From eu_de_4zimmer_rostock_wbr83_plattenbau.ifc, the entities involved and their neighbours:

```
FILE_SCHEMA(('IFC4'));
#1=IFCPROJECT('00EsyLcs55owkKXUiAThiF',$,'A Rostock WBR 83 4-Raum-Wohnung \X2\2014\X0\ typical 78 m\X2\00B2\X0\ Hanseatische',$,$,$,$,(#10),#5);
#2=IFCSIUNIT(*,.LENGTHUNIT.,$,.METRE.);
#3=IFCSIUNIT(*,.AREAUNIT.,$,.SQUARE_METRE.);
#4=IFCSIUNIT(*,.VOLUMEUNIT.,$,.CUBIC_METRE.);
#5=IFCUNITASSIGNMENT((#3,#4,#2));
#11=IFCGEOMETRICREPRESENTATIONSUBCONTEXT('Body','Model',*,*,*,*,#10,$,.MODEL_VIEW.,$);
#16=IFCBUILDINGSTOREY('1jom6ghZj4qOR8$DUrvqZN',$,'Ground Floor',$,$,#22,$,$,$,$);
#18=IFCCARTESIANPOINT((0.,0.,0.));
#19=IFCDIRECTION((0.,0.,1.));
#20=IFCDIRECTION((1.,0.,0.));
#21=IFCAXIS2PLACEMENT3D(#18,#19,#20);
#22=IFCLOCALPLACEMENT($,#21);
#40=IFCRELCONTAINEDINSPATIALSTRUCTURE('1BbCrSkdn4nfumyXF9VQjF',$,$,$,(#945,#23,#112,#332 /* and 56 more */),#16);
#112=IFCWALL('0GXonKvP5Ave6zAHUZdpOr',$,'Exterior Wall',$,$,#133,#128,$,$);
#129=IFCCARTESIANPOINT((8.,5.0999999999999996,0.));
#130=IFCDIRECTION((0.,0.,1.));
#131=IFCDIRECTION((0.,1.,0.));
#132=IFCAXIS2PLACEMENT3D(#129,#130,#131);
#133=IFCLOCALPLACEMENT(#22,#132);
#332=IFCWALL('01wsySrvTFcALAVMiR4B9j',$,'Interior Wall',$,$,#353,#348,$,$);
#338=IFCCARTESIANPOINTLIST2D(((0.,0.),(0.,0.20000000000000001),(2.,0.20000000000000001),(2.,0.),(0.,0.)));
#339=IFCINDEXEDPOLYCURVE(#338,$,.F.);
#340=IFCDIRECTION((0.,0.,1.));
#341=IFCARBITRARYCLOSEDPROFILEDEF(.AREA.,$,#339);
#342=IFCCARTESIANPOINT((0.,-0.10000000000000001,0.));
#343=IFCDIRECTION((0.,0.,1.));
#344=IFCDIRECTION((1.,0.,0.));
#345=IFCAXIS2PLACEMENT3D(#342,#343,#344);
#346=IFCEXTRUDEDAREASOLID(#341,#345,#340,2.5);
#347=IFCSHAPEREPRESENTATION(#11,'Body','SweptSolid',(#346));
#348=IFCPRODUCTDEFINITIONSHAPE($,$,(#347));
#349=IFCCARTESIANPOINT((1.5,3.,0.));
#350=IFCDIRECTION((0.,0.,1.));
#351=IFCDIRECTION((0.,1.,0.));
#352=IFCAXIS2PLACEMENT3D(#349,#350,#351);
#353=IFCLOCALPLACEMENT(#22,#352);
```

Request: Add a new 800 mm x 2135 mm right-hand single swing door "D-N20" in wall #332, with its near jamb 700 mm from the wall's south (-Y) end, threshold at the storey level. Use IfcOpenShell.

```python
import numpy as np
import ifcopenshell
import ifcopenshell.api.feature
import ifcopenshell.api.geometry
import ifcopenshell.api.root
import ifcopenshell.api.spatial
import ifcopenshell.geom
import ifcopenshell.util.element
import ifcopenshell.util.placement
import ifcopenshell.util.representation
import ifcopenshell.util.shape
import ifcopenshell.util.unit

model = ifcopenshell.open("eu_de_4zimmer_rostock_wbr83_plattenbau.ifc")
unit_scale = ifcopenshell.util.unit.calculate_unit_scale(model)
settings = ifcopenshell.geom.settings()


def volume(element):
    """Net volume in cubic metres, openings subtracted."""
    shape = ifcopenshell.geom.create_shape(settings, element)
    return ifcopenshell.util.shape.get_volume(shape.geometry)


wall = model.by_guid("01wsySrvTFcALAVMiR4B9j")
storey = ifcopenshell.util.element.get_container(wall, ifc_class="IfcBuildingStorey")
context = ifcopenshell.util.representation.get_context(model, "Model", "Body", "MODEL_VIEW")
before = volume(wall)

width, height, from_end, sill = 0.8, 2.135, 0.7, 0.0  # metres

# The wall runs along its own X axis, and the end named is its -X end.
wall_shape = ifcopenshell.geom.create_shape(settings, wall)
x, y, z = ifcopenshell.util.shape.get_vertices(wall_shape.geometry).T
start = x.min() + from_end
face, thickness = float(y.min()), float(y.max() - y.min())
wall_matrix = ifcopenshell.util.placement.get_local_placement(wall.ObjectPlacement)
level = ifcopenshell.util.placement.get_local_placement(storey.ObjectPlacement)[2, 3]


def in_wall(x, y):
    """Placement at x, y metres in the wall's axes, at sill height."""
    matrix = wall_matrix.copy()
    matrix[:, 3] = wall_matrix @ np.array([x / unit_scale, y / unit_scale, 0.0, 1.0])
    matrix[2, 3] = level + sill / unit_scale
    return matrix


# Opening: a box that overshoots both wall faces by 50 mm.
opening = ifcopenshell.api.root.create_entity(model, ifc_class="IfcOpeningElement", predefined_type="OPENING")
box = ifcopenshell.api.geometry.add_wall_representation(
    model, context=context, length=width, height=height, thickness=thickness + 0.1
)
ifcopenshell.api.geometry.assign_representation(model, product=opening, representation=box)
ifcopenshell.api.geometry.edit_object_placement(model, product=opening, matrix=in_wall(start, face - 0.05), is_si=False)
ifcopenshell.api.feature.add_feature(model, feature=opening, element=wall)

door = ifcopenshell.api.root.create_entity(model, ifc_class="IfcDoor", name="D-N20", predefined_type="DOOR")
door.OverallWidth, door.OverallHeight = width / unit_scale, height / unit_scale
door.OperationType = "SINGLE_SWING_RIGHT"
body = ifcopenshell.api.geometry.add_door_representation(
    model,
    context=context,
    overall_width=door.OverallWidth,
    overall_height=door.OverallHeight,
    operation_type="SINGLE_SWING_RIGHT",
    lining_properties={"LiningDepth": thickness / unit_scale, "ThresholdDepth": thickness / unit_scale},
)
ifcopenshell.api.geometry.assign_representation(model, product=door, representation=body)
ifcopenshell.api.spatial.assign_container(model, products=[door], relating_structure=storey)
ifcopenshell.api.feature.add_filling(model, opening=opening, element=door)

# The lining spans the wall, so the door starts at the wall face.
ifcopenshell.api.geometry.edit_object_placement(model, product=door, matrix=in_wall(start, face), is_si=False)

after = volume(wall)

print(f"wall volume {before:.3f} -> {after:.3f} m3")

model.write("eu_de_4zimmer_rostock_wbr83_plattenbau_updated.ifc")
```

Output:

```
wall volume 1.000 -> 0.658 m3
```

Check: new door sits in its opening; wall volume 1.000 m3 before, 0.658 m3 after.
